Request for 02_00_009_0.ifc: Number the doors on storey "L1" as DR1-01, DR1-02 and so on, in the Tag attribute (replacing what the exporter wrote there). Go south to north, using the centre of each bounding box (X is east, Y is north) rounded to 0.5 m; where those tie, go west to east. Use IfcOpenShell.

First a look at what the model holds.

```python
import ifcopenshell
import ifcopenshell.util.element
import ifcopenshell.util.placement

model = ifcopenshell.open("02_00_009_0.ifc")
print(model.schema)
storey = next(s for s in model.by_type("IfcBuildingStorey") if s.Name == "L1")
doors = [e for e in ifcopenshell.util.element.get_decomposition(storey) if e.is_a("IfcDoor")]
for e in sorted(doors, key=lambda e: e.id()):
    origin = ifcopenshell.util.placement.get_local_placement(e.ObjectPlacement)[:3, 3]
    print(e.id(), e.Tag, e.Name, origin.round(2) + 0.0, sep=" | ")
```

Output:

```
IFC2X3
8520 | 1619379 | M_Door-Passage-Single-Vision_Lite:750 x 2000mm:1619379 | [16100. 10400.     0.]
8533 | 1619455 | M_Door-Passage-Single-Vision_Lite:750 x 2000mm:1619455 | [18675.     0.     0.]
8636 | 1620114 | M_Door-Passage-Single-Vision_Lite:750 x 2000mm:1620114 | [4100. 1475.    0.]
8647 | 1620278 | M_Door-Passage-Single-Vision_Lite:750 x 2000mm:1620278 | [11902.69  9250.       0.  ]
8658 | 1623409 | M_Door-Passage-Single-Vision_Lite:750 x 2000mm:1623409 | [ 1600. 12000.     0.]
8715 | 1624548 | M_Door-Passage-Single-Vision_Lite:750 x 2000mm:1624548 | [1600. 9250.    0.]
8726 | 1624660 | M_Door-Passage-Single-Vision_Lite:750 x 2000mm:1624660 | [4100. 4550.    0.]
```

```python
import ifcopenshell
import ifcopenshell.geom
import ifcopenshell.util.element
import ifcopenshell.util.shape

model = ifcopenshell.open("02_00_009_0.ifc")
settings = ifcopenshell.geom.settings()
settings.set("use-world-coords", True)


def centre(element):
    shape = ifcopenshell.geom.create_shape(settings, element)
    return ifcopenshell.util.shape.get_bbox_centroid(shape.geometry)


storey = next(s for s in model.by_type("IfcBuildingStorey") if s.Name == "L1")
doors = [e for e in ifcopenshell.util.element.get_decomposition(storey) if e.is_a("IfcDoor")]

# Insertion points can sit at a corner or the storey origin, so sort by the geometry (in metres).
centres = {e: centre(e) for e in doors}
doors.sort(key=lambda e: (round(centres[e][1] / 0.5), centres[e][0]))

for i, e in enumerate(doors, start=1):
    number = f"DR1-{i:02d}"
    e.Tag = number
    print(e.id(), number)

model.write("02_00_009_0_rev.ifc")
```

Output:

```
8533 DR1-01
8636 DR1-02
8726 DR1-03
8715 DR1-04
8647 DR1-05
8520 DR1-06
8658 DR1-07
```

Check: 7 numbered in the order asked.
